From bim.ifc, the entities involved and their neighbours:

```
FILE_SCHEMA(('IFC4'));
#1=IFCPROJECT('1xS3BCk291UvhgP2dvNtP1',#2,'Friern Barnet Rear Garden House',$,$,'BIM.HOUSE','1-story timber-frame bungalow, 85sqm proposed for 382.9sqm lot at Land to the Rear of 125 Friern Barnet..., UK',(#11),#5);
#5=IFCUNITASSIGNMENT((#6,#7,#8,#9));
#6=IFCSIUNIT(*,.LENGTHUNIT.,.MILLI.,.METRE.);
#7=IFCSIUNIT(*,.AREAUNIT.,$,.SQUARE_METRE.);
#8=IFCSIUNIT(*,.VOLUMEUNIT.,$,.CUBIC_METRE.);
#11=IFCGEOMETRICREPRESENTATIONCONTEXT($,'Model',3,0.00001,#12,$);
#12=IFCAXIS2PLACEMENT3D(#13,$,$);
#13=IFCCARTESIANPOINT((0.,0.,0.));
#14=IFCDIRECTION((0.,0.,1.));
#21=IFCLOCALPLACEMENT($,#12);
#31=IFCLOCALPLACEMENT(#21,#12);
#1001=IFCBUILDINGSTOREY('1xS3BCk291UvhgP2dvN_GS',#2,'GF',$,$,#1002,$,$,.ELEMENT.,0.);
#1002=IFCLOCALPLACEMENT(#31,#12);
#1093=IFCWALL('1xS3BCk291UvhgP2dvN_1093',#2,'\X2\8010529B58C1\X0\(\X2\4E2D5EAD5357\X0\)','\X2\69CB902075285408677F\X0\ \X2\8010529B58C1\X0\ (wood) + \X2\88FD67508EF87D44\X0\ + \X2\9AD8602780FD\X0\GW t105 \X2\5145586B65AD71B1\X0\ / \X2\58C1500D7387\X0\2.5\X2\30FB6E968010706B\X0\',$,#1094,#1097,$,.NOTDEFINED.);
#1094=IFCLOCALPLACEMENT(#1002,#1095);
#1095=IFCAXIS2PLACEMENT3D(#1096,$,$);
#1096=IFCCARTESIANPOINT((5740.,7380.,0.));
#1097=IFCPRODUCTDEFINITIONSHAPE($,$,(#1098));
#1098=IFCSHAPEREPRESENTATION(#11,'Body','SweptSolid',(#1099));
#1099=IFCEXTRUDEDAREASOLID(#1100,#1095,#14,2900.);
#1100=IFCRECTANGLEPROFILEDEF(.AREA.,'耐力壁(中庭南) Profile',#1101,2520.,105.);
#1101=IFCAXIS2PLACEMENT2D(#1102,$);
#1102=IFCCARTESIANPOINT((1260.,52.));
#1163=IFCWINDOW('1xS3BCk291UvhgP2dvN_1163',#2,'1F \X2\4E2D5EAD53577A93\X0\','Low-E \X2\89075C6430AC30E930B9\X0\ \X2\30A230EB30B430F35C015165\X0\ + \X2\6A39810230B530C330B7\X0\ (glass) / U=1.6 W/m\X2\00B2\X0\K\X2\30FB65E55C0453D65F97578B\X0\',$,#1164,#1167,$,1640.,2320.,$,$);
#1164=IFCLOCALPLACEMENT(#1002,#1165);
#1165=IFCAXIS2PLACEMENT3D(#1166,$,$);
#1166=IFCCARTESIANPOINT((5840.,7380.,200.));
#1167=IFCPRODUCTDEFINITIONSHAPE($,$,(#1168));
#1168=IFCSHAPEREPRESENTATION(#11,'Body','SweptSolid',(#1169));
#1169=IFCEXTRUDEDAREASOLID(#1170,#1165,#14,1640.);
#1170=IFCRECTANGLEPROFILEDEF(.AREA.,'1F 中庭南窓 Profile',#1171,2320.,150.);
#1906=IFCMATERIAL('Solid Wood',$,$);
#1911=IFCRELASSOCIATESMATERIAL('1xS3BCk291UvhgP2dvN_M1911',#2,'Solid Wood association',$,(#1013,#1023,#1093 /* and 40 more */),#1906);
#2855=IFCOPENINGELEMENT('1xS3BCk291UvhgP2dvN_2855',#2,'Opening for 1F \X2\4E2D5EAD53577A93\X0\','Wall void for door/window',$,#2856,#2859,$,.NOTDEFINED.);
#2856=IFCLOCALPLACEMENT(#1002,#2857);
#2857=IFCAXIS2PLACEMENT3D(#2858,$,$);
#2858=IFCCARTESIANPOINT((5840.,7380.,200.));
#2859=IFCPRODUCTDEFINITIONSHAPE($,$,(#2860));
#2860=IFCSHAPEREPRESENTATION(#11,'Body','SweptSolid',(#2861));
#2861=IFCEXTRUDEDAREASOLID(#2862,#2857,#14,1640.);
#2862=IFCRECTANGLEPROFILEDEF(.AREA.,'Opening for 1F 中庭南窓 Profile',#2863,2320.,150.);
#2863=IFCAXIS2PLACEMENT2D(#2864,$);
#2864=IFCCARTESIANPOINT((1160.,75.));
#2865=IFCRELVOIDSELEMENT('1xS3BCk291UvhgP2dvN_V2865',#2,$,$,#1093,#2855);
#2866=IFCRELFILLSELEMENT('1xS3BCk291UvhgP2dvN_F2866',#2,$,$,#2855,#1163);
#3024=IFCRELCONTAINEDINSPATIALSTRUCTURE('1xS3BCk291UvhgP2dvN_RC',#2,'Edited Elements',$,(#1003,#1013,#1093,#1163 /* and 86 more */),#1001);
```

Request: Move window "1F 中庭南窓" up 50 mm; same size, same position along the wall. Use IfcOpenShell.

```python
import numpy as np
import ifcopenshell
import ifcopenshell.api.geometry
import ifcopenshell.util.placement
import ifcopenshell.util.unit

model = ifcopenshell.open("bim.ifc")
unit_scale = ifcopenshell.util.unit.calculate_unit_scale(model)

window = model.by_id(1163)
opening = window.FillsVoids[0].RelatingOpeningElement
dz = 50.0

shift = np.array([0.0, 0.0, dz])
# The window is not placed relative to its opening, so move both.
for product in (opening, window):
    matrix = ifcopenshell.util.placement.get_local_placement(product.ObjectPlacement)
    matrix[:3, 3] += shift
    ifcopenshell.api.geometry.edit_object_placement(model, product=product, matrix=matrix, is_si=False)

print(f"moved by {dz * unit_scale:+.3f} m")

model.write("bim-out.ifc")
```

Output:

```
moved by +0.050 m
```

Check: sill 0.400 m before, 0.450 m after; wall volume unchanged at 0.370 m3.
